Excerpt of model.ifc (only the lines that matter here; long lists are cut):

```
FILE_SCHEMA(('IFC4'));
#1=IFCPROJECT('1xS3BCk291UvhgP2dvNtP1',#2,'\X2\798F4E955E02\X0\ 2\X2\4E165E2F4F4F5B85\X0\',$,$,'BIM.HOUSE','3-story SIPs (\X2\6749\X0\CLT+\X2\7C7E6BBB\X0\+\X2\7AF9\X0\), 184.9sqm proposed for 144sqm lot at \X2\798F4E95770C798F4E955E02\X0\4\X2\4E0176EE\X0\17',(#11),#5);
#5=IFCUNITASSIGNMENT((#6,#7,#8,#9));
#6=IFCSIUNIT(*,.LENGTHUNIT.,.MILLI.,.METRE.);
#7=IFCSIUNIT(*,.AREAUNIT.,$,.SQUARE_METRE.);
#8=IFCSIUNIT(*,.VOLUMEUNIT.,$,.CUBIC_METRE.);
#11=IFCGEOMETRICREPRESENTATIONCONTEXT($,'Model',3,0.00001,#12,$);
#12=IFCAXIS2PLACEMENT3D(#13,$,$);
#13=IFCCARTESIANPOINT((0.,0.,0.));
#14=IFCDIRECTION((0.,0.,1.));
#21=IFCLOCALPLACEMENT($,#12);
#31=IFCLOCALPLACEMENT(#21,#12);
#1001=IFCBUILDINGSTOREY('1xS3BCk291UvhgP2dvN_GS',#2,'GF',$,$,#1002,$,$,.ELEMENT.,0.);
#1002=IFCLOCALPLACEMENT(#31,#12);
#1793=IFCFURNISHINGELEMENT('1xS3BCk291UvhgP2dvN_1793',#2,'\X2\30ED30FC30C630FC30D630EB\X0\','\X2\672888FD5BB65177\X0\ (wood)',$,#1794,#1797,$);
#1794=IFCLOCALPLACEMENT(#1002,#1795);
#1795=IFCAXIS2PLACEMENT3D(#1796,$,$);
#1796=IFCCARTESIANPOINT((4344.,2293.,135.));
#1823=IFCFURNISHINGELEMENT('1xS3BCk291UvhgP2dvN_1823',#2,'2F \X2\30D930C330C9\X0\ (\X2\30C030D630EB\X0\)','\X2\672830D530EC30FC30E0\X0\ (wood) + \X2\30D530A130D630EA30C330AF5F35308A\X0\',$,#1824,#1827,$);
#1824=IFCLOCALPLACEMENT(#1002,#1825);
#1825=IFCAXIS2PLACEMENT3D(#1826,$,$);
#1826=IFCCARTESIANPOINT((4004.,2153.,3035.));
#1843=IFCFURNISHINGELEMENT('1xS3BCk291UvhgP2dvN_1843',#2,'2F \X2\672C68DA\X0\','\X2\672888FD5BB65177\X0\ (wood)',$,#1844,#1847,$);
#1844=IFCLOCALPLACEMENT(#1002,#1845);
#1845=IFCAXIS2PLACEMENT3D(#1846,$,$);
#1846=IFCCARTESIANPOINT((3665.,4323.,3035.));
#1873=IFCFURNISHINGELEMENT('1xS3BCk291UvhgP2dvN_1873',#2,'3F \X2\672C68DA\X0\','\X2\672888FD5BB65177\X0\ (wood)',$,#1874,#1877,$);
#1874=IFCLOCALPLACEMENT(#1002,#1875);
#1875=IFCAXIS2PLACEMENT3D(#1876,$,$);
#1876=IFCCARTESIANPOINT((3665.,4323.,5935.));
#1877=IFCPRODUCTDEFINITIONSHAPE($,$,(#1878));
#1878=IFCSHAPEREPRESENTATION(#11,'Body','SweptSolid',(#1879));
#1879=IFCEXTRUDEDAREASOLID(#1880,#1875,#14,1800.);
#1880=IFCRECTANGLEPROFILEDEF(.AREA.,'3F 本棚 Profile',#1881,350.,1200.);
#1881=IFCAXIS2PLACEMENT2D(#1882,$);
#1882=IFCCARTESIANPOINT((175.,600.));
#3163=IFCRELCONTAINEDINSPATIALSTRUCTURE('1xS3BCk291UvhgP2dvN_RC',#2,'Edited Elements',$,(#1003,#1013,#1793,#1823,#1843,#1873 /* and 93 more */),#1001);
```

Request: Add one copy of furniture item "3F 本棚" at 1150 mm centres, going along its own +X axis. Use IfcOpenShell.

```python
import ifcopenshell
import ifcopenshell.api.geometry
import ifcopenshell.api.root
import ifcopenshell.util.element
import ifcopenshell.util.placement
import ifcopenshell.util.unit

model = ifcopenshell.open("model.ifc")
unit_scale = ifcopenshell.util.unit.calculate_unit_scale(model)


def reuse_history(source, copy):
    """copy_class also copies each property set's owner history, people and application; keep the originals."""
    for rel in copy.IsDefinedBy:
        if rel.is_a("IfcRelDefinesByProperties") and (history := rel.RelatingPropertyDefinition.OwnerHistory):
            rel.RelatingPropertyDefinition.OwnerHistory = source.OwnerHistory
            ifcopenshell.util.element.remove_deep2(model, history)


source = model.by_guid("1xS3BCk291UvhgP2dvN_1873")
base = ifcopenshell.util.placement.get_local_placement(source.ObjectPlacement)
step = base[:3, 0] * 1.15 / unit_scale

for i in range(1, 2):
    copy = ifcopenshell.api.root.copy_class(model, product=source)
    copy.Representation = ifcopenshell.util.element.copy_deep(
        model, source.Representation, exclude=["IfcGeometricRepresentationContext", "IfcRepresentationMap"]
    )
    reuse_history(source, copy)
    matrix = base.copy()
    matrix[:3, 3] += i * step
    print("added at", matrix[:3, 3].round(3) + 0.0)
    ifcopenshell.api.geometry.edit_object_placement(model, product=copy, matrix=matrix, is_si=False)

model.write("model_rev.ifc")
```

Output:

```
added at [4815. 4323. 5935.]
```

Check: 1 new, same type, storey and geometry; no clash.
